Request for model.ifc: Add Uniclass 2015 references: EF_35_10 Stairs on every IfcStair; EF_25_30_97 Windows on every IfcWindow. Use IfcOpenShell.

First a look at what the model holds.

```python
import ifcopenshell

model = ifcopenshell.open("model.ifc")
print(model.schema)
print("classifications:", [c.Name for c in model.by_type("IfcClassification")])
for ifc_class in ("IfcDoor", "IfcRoof", "IfcStair", "IfcWall", "IfcWindow"):
    print(ifc_class, len(model.by_type(ifc_class)))
```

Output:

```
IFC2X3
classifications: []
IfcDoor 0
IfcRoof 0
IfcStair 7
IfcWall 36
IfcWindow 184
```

```python
import ifcopenshell
import ifcopenshell.api.classification

model = ifcopenshell.open("model.ifc")

# IFC2X3 requires Source and Edition and has no link from the project to the system.
system = model.create_entity("IfcClassification", Source="NBS", Edition="2015", Name="Uniclass 2015")

codes = {
    "IfcStair": ("EF_35_10", "Stairs"),
    "IfcWindow": ("EF_25_30_97", "Windows"),
}
for ifc_class, (code, name) in codes.items():
    products = model.by_type(ifc_class)
    ifcopenshell.api.classification.add_reference(
        model, products=products, classification=system, identification=code, name=name
    )
    print(code, len(products))

model.write("model_rev.ifc")
```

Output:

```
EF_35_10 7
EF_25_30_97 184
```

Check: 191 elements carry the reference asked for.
